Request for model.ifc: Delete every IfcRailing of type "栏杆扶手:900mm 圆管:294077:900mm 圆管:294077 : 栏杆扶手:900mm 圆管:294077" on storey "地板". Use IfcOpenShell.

First a look at what the model holds.

```python
import ifcopenshell
import ifcopenshell.util.element

model = ifcopenshell.open("model.ifc")
print(model.schema)
storey = next(s for s in model.by_type("IfcBuildingStorey") if s.Name == "地板")
railings = [e for e in ifcopenshell.util.element.get_decomposition(storey) if e.is_a("IfcRailing")]
seen = {}
for e in railings:
    element_type = ifcopenshell.util.element.get_type(e)
    name = element_type.Name if element_type not in (None, e) else None
    seen[name] = seen.get(name, 0) + 1
for name, count in sorted(seen.items(), key=str):
    print(count, "x", name)
```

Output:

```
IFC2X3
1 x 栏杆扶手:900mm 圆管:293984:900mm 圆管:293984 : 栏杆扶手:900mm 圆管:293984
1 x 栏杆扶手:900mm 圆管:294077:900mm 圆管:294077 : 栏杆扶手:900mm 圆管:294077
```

```python
import ifcopenshell
import ifcopenshell.api.root
import ifcopenshell.util.element

model = ifcopenshell.open("model.ifc")

storey = next(s for s in model.by_type("IfcBuildingStorey") if s.Name == "地板")
railings = [e for e in ifcopenshell.util.element.get_decomposition(storey) if e.is_a("IfcRailing")]
targets = [e for e in railings if (t := ifcopenshell.util.element.get_type(e)) not in (None, e) and t.Name == "栏杆扶手:900mm 圆管:294077:900mm 圆管:294077 : 栏杆扶手:900mm 圆管:294077"]

for e in targets:
    ifcopenshell.api.root.remove_product(model, product=e)
print(len(targets), "removed")

model.write("model_updated.ifc")
```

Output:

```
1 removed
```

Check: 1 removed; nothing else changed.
